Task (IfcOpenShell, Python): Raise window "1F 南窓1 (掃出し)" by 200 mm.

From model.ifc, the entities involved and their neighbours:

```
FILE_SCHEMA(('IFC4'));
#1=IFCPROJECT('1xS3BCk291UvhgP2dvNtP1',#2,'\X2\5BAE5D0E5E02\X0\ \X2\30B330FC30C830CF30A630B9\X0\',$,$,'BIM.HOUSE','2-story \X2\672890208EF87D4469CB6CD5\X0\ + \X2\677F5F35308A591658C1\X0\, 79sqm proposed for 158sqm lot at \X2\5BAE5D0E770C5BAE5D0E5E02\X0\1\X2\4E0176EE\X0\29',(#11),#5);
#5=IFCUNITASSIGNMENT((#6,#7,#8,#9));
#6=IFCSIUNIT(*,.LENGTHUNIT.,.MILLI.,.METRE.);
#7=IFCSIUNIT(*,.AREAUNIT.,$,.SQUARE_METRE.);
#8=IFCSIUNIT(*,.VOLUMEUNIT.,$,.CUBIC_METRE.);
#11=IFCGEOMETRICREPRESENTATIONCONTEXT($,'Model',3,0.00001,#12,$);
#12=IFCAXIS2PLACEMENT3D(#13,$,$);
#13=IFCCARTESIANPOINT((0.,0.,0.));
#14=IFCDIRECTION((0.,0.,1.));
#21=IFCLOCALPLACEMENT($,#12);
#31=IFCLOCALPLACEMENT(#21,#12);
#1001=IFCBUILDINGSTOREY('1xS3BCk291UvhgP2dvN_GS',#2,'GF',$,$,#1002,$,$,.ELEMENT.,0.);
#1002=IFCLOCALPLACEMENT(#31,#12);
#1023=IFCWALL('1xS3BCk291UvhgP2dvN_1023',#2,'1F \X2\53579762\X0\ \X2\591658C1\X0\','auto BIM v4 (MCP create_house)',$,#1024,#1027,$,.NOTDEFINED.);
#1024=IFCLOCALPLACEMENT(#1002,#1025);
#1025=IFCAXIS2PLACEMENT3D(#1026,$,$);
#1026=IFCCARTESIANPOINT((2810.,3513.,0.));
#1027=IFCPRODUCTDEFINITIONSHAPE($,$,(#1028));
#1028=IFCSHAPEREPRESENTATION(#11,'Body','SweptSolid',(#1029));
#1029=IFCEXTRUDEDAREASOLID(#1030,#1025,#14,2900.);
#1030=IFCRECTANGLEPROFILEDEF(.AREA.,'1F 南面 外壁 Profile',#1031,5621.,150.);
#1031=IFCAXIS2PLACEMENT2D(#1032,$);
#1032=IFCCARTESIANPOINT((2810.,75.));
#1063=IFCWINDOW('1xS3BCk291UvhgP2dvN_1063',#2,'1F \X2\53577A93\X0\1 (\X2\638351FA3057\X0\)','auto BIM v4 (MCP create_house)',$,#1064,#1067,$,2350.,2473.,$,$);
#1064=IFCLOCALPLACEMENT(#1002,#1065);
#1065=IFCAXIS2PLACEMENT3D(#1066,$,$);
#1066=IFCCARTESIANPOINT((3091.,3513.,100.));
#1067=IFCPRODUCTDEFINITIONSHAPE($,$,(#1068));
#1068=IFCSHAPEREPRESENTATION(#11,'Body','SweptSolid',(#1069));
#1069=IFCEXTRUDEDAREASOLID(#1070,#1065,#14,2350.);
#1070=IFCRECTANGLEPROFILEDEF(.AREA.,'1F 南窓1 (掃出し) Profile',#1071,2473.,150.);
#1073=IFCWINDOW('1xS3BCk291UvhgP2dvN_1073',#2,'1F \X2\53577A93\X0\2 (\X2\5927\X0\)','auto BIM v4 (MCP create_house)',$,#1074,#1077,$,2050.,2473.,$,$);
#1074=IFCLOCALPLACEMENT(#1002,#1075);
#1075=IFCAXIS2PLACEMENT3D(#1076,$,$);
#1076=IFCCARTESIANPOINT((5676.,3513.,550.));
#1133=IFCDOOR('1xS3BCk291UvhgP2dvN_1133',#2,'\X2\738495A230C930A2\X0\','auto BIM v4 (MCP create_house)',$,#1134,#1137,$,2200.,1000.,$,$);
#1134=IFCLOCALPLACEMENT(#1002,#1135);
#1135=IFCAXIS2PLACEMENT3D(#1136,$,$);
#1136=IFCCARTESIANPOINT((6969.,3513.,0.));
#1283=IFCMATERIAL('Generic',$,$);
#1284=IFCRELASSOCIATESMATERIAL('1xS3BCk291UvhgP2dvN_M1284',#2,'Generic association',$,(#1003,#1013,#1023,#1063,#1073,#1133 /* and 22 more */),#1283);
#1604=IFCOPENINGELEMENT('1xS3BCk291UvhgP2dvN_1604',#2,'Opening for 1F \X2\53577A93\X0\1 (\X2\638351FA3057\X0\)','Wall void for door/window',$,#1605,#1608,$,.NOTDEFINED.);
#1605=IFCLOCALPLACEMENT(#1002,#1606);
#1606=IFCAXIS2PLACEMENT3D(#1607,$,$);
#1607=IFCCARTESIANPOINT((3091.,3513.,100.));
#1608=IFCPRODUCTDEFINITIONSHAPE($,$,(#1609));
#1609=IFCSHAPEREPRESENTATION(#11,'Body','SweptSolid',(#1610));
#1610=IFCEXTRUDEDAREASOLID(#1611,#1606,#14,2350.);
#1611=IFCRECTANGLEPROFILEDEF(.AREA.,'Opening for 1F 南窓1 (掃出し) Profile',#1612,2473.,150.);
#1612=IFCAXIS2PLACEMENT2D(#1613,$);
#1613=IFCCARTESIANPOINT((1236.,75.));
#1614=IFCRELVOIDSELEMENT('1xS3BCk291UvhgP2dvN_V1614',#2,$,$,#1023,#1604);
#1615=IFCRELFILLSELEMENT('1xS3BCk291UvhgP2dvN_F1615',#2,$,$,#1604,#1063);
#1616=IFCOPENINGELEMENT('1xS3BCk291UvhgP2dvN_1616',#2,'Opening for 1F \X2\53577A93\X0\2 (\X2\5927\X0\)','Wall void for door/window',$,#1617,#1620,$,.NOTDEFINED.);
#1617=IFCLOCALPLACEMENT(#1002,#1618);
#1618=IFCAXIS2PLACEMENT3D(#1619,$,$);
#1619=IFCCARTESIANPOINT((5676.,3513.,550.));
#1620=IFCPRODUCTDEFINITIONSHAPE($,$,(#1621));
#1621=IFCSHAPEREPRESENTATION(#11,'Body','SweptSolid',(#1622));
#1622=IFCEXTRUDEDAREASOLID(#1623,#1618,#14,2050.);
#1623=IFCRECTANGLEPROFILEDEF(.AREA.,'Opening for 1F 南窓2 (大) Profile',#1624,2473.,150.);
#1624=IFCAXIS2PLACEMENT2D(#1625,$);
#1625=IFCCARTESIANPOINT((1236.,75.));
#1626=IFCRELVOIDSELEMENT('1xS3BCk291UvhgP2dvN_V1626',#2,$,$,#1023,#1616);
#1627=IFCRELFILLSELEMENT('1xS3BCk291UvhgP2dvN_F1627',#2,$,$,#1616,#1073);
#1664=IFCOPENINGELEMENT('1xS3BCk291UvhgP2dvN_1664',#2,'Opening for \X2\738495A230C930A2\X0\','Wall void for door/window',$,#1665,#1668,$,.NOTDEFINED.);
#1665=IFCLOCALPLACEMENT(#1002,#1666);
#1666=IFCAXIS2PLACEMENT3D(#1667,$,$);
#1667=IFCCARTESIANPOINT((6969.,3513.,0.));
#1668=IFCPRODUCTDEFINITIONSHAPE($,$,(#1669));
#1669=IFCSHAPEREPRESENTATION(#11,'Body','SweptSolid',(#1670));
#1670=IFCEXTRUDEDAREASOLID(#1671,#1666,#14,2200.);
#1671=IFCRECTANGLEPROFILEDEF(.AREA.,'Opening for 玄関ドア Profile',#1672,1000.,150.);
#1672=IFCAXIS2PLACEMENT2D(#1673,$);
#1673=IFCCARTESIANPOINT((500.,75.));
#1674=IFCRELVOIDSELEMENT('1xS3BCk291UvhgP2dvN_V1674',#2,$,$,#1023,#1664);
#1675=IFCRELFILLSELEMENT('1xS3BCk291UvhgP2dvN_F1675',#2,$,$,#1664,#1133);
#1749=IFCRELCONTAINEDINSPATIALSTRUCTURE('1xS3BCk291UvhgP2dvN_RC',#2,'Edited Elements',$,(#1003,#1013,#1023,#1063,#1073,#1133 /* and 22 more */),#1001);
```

```python
import numpy as np
import ifcopenshell
import ifcopenshell.api.geometry
import ifcopenshell.util.placement
import ifcopenshell.util.unit

model = ifcopenshell.open("model.ifc")
unit_scale = ifcopenshell.util.unit.calculate_unit_scale(model)

window = model.by_id(1063)
opening = window.FillsVoids[0].RelatingOpeningElement
dz = 0.2 / unit_scale

shift = np.array([0.0, 0.0, dz])
# The window is not placed relative to its opening, so move both.
for product in (opening, window):
    matrix = ifcopenshell.util.placement.get_local_placement(product.ObjectPlacement)
    matrix[:3, 3] += shift
    ifcopenshell.api.geometry.edit_object_placement(model, product=product, matrix=matrix, is_si=False)

print(f"moved by {dz * unit_scale:+.3f} m")

model.write("model_rev.ifc")
```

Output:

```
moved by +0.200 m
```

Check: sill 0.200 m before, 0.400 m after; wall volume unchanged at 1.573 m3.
